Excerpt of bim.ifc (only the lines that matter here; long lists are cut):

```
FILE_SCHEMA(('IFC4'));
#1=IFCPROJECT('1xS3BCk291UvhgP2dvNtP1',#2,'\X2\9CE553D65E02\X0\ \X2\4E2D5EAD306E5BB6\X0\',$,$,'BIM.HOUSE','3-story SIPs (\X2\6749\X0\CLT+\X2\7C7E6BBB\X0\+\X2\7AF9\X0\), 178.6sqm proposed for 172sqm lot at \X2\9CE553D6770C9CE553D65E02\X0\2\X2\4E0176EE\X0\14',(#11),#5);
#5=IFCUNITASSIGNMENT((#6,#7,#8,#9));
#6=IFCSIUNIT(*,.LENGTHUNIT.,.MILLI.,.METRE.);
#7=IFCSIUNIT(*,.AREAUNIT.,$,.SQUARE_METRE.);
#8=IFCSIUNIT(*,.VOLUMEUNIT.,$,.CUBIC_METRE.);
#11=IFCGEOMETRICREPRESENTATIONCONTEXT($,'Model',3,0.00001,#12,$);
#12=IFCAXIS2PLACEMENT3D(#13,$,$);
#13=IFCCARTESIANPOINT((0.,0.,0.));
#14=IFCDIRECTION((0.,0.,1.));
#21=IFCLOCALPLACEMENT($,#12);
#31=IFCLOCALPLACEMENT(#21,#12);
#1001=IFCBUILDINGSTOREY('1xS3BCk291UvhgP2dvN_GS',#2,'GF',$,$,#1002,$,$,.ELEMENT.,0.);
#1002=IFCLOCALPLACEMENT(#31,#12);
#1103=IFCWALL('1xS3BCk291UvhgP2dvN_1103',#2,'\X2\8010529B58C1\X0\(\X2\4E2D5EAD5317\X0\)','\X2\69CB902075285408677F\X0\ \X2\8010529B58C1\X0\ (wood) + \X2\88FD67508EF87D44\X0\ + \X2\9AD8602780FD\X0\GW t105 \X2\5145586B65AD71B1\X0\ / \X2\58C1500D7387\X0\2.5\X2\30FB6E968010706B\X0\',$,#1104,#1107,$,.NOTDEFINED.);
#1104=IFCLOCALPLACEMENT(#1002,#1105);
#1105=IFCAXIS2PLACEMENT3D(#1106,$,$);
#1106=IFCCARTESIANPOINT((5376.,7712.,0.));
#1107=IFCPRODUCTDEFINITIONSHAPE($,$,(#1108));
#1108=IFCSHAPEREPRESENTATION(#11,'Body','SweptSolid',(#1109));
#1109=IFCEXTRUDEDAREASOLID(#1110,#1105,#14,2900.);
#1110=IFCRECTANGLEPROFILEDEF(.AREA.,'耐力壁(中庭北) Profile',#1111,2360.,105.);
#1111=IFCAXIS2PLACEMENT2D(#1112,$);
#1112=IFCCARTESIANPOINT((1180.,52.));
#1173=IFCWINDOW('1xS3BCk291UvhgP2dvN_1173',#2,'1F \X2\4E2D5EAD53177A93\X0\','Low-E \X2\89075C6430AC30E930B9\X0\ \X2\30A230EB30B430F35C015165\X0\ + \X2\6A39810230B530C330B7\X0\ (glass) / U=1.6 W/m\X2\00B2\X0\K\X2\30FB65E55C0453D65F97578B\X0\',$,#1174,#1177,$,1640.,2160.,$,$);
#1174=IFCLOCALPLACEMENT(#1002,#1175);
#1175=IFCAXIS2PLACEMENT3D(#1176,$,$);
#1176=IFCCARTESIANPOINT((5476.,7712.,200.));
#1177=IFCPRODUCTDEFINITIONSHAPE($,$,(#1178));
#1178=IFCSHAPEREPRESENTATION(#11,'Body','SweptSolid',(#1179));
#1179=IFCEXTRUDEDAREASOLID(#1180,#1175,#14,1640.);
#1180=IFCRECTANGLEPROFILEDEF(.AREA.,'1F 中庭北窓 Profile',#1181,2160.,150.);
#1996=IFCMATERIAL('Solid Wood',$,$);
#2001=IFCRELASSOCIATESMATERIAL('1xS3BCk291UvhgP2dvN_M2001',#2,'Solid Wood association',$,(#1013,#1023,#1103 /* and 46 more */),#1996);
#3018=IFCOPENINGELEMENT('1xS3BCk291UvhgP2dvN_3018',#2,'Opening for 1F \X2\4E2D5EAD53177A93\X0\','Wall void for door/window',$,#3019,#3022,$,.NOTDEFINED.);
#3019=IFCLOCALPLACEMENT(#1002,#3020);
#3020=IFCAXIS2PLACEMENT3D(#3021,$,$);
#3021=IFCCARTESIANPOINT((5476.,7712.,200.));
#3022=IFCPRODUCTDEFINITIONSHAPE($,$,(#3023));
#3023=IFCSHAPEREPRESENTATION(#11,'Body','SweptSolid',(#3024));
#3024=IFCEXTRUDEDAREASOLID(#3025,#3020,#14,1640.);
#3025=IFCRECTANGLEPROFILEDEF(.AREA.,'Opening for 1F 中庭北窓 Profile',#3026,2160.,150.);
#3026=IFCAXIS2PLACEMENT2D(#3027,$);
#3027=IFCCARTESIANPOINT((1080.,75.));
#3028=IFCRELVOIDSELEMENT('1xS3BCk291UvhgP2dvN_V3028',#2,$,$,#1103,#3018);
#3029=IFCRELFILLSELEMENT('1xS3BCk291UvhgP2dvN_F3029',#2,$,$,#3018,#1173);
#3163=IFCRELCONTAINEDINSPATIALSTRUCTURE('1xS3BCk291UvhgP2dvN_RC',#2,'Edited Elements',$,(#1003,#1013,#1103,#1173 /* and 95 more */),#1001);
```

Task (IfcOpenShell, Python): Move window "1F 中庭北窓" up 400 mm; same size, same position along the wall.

```python
import numpy as np
import ifcopenshell
import ifcopenshell.api.geometry
import ifcopenshell.util.placement
import ifcopenshell.util.unit

model = ifcopenshell.open("bim.ifc")
unit_scale = ifcopenshell.util.unit.calculate_unit_scale(model)

window = model.by_id(1173)
opening = window.FillsVoids[0].RelatingOpeningElement
dz = 0.4 / unit_scale

shift = np.array([0.0, 0.0, dz])
# The window is not placed relative to its opening, so move both.
for product in (opening, window):
    matrix = ifcopenshell.util.placement.get_local_placement(product.ObjectPlacement)
    matrix[:3, 3] += shift
    ifcopenshell.api.geometry.edit_object_placement(model, product=product, matrix=matrix, is_si=False)

print(f"moved by {dz * unit_scale:+.3f} m")

model.write("bim_rev.ifc")
```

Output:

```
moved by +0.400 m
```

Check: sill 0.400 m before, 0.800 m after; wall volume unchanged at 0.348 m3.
